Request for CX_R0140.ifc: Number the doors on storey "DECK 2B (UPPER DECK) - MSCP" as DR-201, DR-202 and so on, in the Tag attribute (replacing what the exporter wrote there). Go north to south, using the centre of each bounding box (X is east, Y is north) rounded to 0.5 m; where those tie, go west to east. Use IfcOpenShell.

First a look at what the model holds.

```python
import ifcopenshell
import ifcopenshell.util.element
import ifcopenshell.util.placement

model = ifcopenshell.open("CX_R0140.ifc")
print(model.schema)
storey = next(s for s in model.by_type("IfcBuildingStorey") if s.Name == "DECK 2B (UPPER DECK) - MSCP")
doors = [e for e in ifcopenshell.util.element.get_decomposition(storey) if e.is_a("IfcDoor")]
for e in sorted(doors, key=lambda e: e.id()):
    origin = ifcopenshell.util.placement.get_local_placement(e.ObjectPlacement)[:3, 3]
    print(e.id(), e.Tag, e.Name, origin.round(2) + 0.0, sep=" | ")
```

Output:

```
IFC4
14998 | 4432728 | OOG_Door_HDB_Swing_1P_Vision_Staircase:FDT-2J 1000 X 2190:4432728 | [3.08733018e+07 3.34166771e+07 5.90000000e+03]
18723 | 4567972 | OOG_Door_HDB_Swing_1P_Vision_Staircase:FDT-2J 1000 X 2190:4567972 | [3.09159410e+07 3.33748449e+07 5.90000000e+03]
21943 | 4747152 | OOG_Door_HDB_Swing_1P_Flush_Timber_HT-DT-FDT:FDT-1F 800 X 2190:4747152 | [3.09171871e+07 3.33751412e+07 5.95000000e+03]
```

```python
import ifcopenshell
import ifcopenshell.geom
import ifcopenshell.util.element
import ifcopenshell.util.shape

model = ifcopenshell.open("CX_R0140.ifc")
settings = ifcopenshell.geom.settings()
settings.set("use-world-coords", True)


def centre(element):
    shape = ifcopenshell.geom.create_shape(settings, element)
    return ifcopenshell.util.shape.get_bbox_centroid(shape.geometry)


storey = next(s for s in model.by_type("IfcBuildingStorey") if s.Name == "DECK 2B (UPPER DECK) - MSCP")
doors = [e for e in ifcopenshell.util.element.get_decomposition(storey) if e.is_a("IfcDoor")]

# Insertion points can sit at a corner or the storey origin, so sort by the geometry (in metres).
centres = {e: centre(e) for e in doors}
doors.sort(key=lambda e: (-round(centres[e][1] / 0.5), centres[e][0]))

for i, e in enumerate(doors, start=1):
    number = f"DR-2{i:02d}"
    e.Tag = number
    print(e.id(), number)

model.write("CX_R0140_updated.ifc")
```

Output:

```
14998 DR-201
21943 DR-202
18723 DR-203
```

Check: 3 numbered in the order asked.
